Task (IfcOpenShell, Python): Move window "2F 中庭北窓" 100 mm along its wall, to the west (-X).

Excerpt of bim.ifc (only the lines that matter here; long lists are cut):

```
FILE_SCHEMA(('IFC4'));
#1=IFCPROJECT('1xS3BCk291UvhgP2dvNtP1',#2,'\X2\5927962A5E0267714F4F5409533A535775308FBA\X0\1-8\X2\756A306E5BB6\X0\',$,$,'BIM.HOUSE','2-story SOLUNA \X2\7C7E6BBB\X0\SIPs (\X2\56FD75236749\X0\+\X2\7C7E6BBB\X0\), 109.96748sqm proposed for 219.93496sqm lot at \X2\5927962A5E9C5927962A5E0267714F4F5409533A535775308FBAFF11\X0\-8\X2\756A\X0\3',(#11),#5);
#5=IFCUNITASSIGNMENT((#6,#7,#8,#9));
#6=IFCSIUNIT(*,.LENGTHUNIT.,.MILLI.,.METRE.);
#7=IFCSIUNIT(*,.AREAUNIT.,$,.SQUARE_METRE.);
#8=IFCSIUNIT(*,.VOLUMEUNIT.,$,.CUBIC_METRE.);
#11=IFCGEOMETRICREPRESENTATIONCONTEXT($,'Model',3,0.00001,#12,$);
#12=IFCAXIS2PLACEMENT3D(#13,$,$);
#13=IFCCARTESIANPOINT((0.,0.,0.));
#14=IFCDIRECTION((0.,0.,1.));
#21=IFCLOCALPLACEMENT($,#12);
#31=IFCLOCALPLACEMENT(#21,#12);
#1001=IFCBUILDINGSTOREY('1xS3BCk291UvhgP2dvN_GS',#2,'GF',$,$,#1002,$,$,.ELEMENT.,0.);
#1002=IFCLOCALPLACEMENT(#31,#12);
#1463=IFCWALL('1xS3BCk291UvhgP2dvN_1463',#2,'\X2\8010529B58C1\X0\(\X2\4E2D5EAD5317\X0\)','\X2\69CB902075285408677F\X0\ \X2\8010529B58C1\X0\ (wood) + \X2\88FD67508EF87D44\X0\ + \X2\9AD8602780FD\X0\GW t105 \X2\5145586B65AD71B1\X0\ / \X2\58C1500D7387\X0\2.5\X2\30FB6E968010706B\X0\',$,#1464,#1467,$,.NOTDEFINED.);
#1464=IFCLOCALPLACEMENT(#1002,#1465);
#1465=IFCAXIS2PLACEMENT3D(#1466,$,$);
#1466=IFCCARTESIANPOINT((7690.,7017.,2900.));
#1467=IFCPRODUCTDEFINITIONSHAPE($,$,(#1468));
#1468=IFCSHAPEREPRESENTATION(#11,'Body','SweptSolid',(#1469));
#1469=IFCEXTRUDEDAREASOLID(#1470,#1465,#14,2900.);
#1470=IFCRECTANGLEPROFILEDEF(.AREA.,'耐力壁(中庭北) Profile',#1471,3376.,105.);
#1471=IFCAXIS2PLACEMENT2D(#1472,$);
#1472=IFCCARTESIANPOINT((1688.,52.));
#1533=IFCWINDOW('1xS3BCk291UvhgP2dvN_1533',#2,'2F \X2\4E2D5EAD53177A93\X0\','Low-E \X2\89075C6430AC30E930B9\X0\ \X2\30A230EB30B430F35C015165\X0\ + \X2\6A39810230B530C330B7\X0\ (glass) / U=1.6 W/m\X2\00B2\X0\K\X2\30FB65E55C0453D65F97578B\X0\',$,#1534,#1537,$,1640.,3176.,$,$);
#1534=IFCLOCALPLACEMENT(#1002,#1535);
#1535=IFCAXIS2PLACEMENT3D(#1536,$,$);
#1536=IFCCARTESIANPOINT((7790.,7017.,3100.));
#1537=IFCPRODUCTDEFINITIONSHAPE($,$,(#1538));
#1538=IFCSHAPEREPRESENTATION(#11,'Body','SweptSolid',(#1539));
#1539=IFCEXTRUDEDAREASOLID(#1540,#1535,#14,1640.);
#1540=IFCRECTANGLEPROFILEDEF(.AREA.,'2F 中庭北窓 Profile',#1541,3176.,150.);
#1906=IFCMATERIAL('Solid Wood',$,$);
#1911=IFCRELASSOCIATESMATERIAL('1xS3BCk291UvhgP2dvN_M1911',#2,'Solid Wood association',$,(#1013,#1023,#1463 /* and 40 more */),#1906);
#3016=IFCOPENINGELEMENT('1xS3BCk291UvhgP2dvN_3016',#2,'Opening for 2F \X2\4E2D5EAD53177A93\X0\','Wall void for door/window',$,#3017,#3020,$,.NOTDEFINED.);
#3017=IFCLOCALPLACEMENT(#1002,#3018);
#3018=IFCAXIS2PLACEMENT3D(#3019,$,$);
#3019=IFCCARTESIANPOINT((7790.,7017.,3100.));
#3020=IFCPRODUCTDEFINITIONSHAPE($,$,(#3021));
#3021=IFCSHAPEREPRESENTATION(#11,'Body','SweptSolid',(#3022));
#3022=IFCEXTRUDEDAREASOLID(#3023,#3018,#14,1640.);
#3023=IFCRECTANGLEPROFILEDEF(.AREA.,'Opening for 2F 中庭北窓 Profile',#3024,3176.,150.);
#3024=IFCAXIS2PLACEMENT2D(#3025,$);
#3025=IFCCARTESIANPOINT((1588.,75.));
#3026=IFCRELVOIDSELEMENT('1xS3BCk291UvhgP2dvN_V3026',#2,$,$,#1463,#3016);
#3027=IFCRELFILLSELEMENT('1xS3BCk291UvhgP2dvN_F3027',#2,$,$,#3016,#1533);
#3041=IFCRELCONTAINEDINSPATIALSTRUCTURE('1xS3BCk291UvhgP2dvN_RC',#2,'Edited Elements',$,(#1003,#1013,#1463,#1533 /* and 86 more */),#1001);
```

```python
import ifcopenshell
import ifcopenshell.api.geometry
import ifcopenshell.util.placement
import ifcopenshell.util.unit

model = ifcopenshell.open("bim.ifc")
unit_scale = ifcopenshell.util.unit.calculate_unit_scale(model)

window = model.by_guid("1xS3BCk291UvhgP2dvN_1533")
opening = window.FillsVoids[0].RelatingOpeningElement
wall = opening.VoidsElements[0].RelatingBuildingElement

wall_matrix = ifcopenshell.util.placement.get_local_placement(wall.ObjectPlacement)
shift = wall_matrix[:3, 0] * -0.1 / unit_scale
before = ifcopenshell.util.placement.get_local_placement(window.ObjectPlacement)[:3, 3].copy()

# The window is not placed relative to its opening, so move both.
for product in (opening, window):
    matrix = ifcopenshell.util.placement.get_local_placement(product.ObjectPlacement)
    matrix[:3, 3] += shift
    ifcopenshell.api.geometry.edit_object_placement(model, product=product, matrix=matrix, is_si=False)

after = ifcopenshell.util.placement.get_local_placement(window.ObjectPlacement)[:3, 3]
print("window moved by", (after - before).round(3) + 0.0)

model.write("bim_updated.ifc")
```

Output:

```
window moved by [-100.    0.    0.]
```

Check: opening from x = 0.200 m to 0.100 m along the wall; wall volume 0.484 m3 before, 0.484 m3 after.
